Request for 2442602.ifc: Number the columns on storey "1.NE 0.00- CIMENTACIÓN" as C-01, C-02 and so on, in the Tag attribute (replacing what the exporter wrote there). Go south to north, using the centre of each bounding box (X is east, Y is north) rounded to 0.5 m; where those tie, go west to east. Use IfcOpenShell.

First a look at what the model holds.

```python
import ifcopenshell
import ifcopenshell.util.element
import ifcopenshell.util.placement

model = ifcopenshell.open("2442602.ifc")
print(model.schema)
storey = next(s for s in model.by_type("IfcBuildingStorey") if s.Name == "1.NE 0.00- CIMENTACIÓN")
columns = [e for e in ifcopenshell.util.element.get_decomposition(storey) if e.is_a("IfcColumn")]
for e in sorted(columns, key=lambda e: e.id()):
    origin = ifcopenshell.util.placement.get_local_placement(e.ObjectPlacement)[:3, 3]
    print(e.id(), e.Tag, e.Name, origin.round(2) + 0.0, sep=" | ")
```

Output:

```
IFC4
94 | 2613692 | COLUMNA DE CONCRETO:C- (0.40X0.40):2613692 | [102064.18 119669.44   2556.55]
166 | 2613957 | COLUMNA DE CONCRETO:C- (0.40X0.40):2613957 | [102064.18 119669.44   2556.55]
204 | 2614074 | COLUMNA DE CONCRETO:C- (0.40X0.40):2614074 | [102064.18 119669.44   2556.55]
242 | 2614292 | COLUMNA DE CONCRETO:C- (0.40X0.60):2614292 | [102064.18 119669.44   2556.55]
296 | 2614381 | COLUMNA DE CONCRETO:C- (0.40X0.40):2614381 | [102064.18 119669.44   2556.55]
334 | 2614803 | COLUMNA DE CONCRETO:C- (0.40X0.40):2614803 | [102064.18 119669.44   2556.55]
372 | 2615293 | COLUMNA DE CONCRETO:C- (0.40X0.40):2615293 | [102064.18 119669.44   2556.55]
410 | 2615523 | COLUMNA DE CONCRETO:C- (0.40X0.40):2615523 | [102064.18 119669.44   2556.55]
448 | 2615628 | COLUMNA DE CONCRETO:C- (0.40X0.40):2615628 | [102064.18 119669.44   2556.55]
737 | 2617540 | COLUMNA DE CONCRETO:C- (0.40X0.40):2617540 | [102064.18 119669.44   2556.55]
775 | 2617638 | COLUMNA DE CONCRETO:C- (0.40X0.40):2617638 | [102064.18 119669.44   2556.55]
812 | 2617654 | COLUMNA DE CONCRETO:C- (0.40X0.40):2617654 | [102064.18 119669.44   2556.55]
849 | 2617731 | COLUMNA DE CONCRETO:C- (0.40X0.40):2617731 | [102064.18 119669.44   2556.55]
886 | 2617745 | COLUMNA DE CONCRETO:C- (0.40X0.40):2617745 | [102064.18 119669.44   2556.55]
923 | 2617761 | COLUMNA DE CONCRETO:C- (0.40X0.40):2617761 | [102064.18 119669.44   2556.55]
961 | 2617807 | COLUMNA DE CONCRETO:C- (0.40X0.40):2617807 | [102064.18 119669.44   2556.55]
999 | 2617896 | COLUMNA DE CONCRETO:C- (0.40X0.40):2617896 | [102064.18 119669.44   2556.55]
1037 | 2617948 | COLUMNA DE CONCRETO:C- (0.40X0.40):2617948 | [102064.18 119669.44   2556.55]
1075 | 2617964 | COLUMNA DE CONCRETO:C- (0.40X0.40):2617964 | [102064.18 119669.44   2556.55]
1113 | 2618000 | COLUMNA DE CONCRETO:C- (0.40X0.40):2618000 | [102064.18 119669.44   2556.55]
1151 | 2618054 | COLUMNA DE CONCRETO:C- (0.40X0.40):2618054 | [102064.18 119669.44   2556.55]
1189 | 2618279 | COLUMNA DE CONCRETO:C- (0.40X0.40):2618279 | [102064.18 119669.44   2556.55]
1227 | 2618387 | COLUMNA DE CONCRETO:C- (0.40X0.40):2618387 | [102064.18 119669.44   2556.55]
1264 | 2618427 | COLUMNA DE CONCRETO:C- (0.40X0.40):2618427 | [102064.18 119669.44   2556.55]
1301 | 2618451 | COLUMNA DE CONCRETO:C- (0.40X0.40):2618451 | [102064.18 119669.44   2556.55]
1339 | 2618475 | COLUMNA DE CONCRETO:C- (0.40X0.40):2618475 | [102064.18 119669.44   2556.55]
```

```python
import ifcopenshell
import ifcopenshell.geom
import ifcopenshell.util.element
import ifcopenshell.util.shape

model = ifcopenshell.open("2442602.ifc")
settings = ifcopenshell.geom.settings()
settings.set("use-world-coords", True)


def centre(element):
    shape = ifcopenshell.geom.create_shape(settings, element)
    return ifcopenshell.util.shape.get_bbox_centroid(shape.geometry)


storey = next(s for s in model.by_type("IfcBuildingStorey") if s.Name == "1.NE 0.00- CIMENTACIÓN")
columns = [e for e in ifcopenshell.util.element.get_decomposition(storey) if e.is_a("IfcColumn")]

# Insertion points can sit at a corner or the storey origin, so sort by the geometry (in metres).
centres = {e: centre(e) for e in columns}
columns.sort(key=lambda e: (round(centres[e][1] / 0.5), centres[e][0]))

for i, e in enumerate(columns, start=1):
    number = f"C-{i:02d}"
    e.Tag = number
    print(e.id(), number)

model.write("2442602_updated.ifc")
```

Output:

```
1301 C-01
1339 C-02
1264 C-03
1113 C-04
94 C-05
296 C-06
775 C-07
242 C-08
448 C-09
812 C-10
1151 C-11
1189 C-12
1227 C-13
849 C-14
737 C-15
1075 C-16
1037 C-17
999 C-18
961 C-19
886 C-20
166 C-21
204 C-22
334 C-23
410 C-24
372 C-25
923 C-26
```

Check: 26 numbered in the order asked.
